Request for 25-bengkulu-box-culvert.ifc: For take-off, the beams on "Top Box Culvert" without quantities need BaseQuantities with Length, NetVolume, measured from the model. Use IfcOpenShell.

First a look at what the model holds.

```python
import ifcopenshell
import ifcopenshell.util.element
import ifcopenshell.util.unit

model = ifcopenshell.open("25-bengkulu-box-culvert.ifc")
print(model.schema)
for unit_type in ("LENGTHUNIT", "AREAUNIT", "VOLUMEUNIT"):
    print(unit_type, ifcopenshell.util.unit.calculate_unit_scale(model, unit_type))
storey = next(s for s in model.by_type("IfcBuildingStorey") if s.Name == "Top Box Culvert")
beams = [e for e in ifcopenshell.util.element.get_decomposition(storey) if e.is_a("IfcBeam")]
for e in sorted(beams, key=lambda e: e.id()):
    print(e.id(), e.is_a(), e.Name, list(ifcopenshell.util.element.get_psets(e, qtos_only=True)), sep=" | ")
```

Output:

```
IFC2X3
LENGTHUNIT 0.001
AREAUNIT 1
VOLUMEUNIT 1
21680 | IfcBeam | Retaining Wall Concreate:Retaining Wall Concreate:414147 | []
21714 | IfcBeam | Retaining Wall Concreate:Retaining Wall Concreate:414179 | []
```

```python
import ifcopenshell
import ifcopenshell.api.pset
import ifcopenshell.geom
import ifcopenshell.util.element
import ifcopenshell.util.shape
import ifcopenshell.util.unit

model = ifcopenshell.open("25-bengkulu-box-culvert.ifc")
unit_scale = ifcopenshell.util.unit.calculate_unit_scale(model)
volume_scale = ifcopenshell.util.unit.calculate_unit_scale(model, "VOLUMEUNIT")
settings = ifcopenshell.geom.settings()

storey = next(s for s in model.by_type("IfcBuildingStorey") if s.Name == "Top Box Culvert")
beams = [e for e in ifcopenshell.util.element.get_decomposition(storey) if e.is_a("IfcBeam")]

for e in sorted(beams, key=lambda e: e.id()):
    if ifcopenshell.util.element.get_psets(e, qtos_only=True, should_inherit=False):
        continue
    # Geometry comes back in metres, in the element's own axes.
    shape = ifcopenshell.geom.create_shape(settings, e)
    values = {
        "Length": ifcopenshell.util.shape.get_max_xyz(shape.geometry) / unit_scale,
        "NetVolume": ifcopenshell.util.shape.get_volume(shape.geometry) / volume_scale,
    }
    qto = ifcopenshell.api.pset.add_qto(model, product=e, name="BaseQuantities")
    ifcopenshell.api.pset.edit_qto(model, qto=qto, properties=values)
    print(e.id(), {k: round(v, 3) for k, v in values.items()})

model.write("25-bengkulu-box-culvert_updated.ifc")
```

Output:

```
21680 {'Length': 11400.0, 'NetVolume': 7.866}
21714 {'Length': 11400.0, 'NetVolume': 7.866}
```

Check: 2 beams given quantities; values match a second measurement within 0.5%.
